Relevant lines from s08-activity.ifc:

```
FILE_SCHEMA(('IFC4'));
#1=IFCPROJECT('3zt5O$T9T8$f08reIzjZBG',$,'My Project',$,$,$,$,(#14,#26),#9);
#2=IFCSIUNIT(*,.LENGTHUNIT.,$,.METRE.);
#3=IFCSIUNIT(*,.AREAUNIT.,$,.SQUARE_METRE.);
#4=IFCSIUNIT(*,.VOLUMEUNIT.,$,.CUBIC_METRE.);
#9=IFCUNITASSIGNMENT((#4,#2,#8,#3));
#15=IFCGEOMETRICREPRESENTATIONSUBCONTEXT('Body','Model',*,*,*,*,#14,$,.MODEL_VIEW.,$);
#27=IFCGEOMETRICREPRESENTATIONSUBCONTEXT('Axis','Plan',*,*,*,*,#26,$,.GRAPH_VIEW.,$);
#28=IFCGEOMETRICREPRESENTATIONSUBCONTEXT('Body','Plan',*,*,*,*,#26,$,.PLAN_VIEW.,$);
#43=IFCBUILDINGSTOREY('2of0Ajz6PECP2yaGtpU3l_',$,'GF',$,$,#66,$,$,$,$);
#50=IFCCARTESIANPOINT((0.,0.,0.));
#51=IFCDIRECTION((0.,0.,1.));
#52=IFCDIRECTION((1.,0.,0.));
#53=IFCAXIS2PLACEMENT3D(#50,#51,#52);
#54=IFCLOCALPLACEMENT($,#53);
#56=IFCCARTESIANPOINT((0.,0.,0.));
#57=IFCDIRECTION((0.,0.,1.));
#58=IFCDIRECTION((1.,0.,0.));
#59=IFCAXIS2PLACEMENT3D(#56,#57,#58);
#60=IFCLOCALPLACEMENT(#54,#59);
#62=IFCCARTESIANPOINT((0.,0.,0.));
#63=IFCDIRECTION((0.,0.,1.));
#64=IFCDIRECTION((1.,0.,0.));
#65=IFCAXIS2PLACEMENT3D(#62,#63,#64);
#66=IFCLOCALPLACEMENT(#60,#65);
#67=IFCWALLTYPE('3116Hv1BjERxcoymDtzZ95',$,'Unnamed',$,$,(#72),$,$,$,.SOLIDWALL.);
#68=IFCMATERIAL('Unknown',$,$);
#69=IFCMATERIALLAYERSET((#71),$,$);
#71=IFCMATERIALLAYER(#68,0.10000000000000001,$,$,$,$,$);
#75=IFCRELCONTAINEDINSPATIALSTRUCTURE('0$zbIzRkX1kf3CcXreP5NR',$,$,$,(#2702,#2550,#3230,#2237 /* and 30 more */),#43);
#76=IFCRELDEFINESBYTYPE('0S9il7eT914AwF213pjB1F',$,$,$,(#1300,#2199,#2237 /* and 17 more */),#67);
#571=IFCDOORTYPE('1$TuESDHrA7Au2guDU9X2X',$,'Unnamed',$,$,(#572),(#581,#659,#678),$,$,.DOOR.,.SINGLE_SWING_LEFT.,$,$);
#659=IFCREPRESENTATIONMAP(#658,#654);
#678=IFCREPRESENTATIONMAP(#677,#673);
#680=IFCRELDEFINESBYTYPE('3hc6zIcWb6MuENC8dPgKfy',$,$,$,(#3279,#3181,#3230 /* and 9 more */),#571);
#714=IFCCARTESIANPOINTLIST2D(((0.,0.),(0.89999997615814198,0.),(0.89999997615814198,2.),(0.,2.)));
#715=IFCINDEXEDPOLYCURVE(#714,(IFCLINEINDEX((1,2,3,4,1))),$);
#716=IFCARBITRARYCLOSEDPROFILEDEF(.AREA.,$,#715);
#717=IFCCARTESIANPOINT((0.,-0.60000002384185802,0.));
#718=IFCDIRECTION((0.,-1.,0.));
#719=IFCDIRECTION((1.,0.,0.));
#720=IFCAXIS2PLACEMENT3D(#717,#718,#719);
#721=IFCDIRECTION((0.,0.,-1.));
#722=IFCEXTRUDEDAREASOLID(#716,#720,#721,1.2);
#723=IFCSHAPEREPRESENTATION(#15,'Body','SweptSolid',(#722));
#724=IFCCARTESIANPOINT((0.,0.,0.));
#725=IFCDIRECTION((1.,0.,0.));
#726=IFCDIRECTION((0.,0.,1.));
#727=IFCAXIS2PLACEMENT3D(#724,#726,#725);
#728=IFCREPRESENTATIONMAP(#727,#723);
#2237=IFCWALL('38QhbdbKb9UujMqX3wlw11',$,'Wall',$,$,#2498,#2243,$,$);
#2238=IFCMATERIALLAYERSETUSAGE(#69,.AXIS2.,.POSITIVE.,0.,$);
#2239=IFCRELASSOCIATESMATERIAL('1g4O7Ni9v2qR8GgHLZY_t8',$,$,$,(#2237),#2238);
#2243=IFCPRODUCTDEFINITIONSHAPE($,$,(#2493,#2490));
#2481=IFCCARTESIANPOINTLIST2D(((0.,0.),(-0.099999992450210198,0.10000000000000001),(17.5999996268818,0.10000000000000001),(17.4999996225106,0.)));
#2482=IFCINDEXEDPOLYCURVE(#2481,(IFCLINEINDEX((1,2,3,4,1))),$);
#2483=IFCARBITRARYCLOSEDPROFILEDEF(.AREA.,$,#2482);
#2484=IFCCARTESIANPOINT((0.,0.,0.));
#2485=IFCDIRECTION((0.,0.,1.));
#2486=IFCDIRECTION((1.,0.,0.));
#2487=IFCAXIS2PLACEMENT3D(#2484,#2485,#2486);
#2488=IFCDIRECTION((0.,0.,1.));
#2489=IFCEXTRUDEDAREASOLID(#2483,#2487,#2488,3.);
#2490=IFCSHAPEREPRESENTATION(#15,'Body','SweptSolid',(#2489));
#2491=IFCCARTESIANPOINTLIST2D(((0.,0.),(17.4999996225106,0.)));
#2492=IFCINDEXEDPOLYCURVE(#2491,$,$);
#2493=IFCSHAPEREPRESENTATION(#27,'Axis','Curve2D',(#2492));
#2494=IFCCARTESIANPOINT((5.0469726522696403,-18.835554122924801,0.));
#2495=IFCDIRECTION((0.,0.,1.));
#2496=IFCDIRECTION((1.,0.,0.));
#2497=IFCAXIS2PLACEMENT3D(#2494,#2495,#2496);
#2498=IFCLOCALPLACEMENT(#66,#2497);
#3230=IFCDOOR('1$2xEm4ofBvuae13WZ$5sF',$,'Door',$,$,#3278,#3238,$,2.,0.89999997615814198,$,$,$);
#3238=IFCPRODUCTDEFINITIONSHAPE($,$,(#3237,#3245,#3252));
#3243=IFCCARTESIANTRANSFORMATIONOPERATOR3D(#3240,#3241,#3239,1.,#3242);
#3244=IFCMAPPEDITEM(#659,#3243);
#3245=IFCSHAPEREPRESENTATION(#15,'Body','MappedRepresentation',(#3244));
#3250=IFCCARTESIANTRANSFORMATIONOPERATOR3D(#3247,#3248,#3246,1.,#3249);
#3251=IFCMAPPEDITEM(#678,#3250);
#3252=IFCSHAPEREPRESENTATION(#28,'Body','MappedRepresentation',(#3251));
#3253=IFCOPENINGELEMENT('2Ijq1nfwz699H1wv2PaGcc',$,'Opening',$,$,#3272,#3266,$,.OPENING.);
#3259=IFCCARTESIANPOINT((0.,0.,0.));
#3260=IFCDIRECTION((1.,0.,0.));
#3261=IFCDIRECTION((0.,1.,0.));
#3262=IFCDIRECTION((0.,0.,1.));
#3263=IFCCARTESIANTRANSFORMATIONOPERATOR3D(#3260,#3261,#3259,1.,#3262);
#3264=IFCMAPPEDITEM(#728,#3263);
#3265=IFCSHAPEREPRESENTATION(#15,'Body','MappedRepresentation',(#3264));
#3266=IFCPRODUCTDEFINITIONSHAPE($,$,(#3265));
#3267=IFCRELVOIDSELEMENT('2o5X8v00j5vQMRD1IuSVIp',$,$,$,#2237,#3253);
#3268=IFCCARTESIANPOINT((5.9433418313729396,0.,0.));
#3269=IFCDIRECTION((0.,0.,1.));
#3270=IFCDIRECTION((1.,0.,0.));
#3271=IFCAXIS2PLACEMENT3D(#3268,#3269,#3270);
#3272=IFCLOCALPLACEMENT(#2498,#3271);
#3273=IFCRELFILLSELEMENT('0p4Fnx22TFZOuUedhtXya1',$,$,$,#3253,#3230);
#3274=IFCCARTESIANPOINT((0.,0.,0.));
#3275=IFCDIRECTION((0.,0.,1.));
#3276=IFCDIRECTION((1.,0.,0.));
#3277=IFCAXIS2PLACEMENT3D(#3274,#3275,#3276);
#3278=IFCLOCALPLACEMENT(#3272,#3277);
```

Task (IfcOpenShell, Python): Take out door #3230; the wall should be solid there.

```python
import ifcopenshell
import ifcopenshell.api.feature
import ifcopenshell.api.root
import ifcopenshell.geom
import ifcopenshell.util.shape

model = ifcopenshell.open("s08-activity.ifc")
settings = ifcopenshell.geom.settings()


def volume(element):
    """Net volume in cubic metres, openings subtracted."""
    shape = ifcopenshell.geom.create_shape(settings, element)
    return ifcopenshell.util.shape.get_volume(shape.geometry)


door = model.by_guid("1$2xEm4ofBvuae13WZ$5sF")
opening = door.FillsVoids[0].RelatingOpeningElement
wall = opening.VoidsElements[0].RelatingBuildingElement
before = volume(wall)

ifcopenshell.api.root.remove_product(model, product=door)
ifcopenshell.api.feature.remove_feature(model, feature=opening)

after = volume(wall)

print(f"wall volume {before:.3f} -> {after:.3f} m3")

model.write("s08-activity_rev.ifc")
```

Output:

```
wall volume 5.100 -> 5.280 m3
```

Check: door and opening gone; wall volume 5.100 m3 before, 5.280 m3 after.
